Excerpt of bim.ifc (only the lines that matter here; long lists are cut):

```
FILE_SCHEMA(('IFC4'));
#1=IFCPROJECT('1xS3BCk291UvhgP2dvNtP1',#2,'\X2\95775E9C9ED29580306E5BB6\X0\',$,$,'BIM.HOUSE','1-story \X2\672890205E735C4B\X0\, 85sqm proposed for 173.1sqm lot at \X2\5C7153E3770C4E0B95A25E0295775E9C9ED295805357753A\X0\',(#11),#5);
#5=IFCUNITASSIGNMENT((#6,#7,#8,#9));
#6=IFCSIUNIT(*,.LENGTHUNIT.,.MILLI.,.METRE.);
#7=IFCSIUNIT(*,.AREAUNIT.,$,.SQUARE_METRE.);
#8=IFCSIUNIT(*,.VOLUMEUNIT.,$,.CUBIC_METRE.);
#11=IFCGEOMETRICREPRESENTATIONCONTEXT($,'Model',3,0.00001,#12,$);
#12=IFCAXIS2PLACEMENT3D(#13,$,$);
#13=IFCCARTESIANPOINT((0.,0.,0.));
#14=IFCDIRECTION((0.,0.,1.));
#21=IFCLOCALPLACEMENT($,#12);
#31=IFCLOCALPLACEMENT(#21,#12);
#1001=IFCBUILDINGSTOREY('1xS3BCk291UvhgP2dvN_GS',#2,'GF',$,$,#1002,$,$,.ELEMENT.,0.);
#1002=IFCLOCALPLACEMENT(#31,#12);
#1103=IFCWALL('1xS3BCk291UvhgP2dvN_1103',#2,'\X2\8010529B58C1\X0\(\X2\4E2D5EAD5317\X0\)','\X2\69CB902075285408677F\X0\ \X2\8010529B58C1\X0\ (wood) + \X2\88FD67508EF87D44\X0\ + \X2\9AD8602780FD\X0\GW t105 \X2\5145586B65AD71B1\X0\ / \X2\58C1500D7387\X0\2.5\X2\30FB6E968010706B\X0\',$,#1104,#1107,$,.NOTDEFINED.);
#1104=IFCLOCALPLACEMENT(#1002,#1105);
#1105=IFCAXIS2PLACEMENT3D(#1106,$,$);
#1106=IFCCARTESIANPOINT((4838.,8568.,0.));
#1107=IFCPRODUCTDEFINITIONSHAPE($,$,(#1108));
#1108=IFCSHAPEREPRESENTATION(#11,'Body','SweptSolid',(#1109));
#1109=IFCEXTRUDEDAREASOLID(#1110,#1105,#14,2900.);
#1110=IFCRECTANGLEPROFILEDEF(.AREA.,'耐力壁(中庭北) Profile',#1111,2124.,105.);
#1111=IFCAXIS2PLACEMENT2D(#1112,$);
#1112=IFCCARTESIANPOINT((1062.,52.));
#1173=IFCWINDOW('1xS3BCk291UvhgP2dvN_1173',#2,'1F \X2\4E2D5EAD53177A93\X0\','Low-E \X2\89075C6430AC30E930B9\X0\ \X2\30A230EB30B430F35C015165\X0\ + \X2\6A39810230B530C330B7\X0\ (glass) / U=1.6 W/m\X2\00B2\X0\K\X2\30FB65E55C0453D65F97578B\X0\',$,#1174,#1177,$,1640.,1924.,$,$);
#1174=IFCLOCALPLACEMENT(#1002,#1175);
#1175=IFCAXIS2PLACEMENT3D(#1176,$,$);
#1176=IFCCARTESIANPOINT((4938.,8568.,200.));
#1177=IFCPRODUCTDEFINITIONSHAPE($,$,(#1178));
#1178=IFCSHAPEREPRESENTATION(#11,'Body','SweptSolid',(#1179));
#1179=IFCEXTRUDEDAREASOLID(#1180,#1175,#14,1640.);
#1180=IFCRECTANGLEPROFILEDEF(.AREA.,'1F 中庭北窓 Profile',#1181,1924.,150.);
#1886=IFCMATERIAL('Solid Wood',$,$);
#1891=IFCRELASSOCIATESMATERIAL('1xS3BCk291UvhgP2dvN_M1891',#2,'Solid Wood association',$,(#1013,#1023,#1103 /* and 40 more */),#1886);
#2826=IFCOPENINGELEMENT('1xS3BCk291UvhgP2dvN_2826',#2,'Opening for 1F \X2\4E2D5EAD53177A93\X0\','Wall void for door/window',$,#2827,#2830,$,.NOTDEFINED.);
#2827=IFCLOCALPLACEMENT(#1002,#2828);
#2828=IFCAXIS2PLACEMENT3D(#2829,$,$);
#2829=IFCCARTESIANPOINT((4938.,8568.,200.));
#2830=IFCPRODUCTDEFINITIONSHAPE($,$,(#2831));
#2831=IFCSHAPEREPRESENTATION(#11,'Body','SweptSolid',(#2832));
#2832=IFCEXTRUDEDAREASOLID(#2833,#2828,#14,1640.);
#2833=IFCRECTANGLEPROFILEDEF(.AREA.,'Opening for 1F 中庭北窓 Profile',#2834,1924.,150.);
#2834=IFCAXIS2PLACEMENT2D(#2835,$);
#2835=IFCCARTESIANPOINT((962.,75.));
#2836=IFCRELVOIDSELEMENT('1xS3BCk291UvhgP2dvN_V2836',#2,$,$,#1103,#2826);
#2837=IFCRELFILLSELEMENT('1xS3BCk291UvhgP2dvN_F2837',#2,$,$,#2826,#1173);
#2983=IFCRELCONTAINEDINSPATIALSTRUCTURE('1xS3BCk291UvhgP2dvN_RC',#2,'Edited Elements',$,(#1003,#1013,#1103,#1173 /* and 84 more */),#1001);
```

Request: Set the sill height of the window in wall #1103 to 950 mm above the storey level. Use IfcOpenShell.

```python
import numpy as np
import ifcopenshell
import ifcopenshell.api.geometry
import ifcopenshell.geom
import ifcopenshell.util.element
import ifcopenshell.util.placement
import ifcopenshell.util.shape
import ifcopenshell.util.unit

model = ifcopenshell.open("bim.ifc")
unit_scale = ifcopenshell.util.unit.calculate_unit_scale(model)

window = model.by_id(1173)
opening = window.FillsVoids[0].RelatingOpeningElement
storey = ifcopenshell.util.element.get_container(window, ifc_class="IfcBuildingStorey")
level = ifcopenshell.util.placement.get_local_placement(storey.ObjectPlacement)[2, 3]

# The opening's origin need not be at the sill, so measure its lowest point.
shape = ifcopenshell.geom.create_shape(ifcopenshell.geom.settings(), opening)
bottom = ifcopenshell.util.shape.get_shape_bottom_elevation(shape, shape.geometry) / unit_scale
dz = level + 0.95 / unit_scale - bottom

shift = np.array([0.0, 0.0, dz])
# The window is not placed relative to its opening, so move both.
for product in (opening, window):
    matrix = ifcopenshell.util.placement.get_local_placement(product.ObjectPlacement)
    matrix[:3, 3] += shift
    ifcopenshell.api.geometry.edit_object_placement(model, product=product, matrix=matrix, is_si=False)

print(f"moved by {dz * unit_scale:+.3f} m")

model.write("bim-out.ifc")
```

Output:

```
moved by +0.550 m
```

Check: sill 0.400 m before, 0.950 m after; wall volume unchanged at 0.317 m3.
